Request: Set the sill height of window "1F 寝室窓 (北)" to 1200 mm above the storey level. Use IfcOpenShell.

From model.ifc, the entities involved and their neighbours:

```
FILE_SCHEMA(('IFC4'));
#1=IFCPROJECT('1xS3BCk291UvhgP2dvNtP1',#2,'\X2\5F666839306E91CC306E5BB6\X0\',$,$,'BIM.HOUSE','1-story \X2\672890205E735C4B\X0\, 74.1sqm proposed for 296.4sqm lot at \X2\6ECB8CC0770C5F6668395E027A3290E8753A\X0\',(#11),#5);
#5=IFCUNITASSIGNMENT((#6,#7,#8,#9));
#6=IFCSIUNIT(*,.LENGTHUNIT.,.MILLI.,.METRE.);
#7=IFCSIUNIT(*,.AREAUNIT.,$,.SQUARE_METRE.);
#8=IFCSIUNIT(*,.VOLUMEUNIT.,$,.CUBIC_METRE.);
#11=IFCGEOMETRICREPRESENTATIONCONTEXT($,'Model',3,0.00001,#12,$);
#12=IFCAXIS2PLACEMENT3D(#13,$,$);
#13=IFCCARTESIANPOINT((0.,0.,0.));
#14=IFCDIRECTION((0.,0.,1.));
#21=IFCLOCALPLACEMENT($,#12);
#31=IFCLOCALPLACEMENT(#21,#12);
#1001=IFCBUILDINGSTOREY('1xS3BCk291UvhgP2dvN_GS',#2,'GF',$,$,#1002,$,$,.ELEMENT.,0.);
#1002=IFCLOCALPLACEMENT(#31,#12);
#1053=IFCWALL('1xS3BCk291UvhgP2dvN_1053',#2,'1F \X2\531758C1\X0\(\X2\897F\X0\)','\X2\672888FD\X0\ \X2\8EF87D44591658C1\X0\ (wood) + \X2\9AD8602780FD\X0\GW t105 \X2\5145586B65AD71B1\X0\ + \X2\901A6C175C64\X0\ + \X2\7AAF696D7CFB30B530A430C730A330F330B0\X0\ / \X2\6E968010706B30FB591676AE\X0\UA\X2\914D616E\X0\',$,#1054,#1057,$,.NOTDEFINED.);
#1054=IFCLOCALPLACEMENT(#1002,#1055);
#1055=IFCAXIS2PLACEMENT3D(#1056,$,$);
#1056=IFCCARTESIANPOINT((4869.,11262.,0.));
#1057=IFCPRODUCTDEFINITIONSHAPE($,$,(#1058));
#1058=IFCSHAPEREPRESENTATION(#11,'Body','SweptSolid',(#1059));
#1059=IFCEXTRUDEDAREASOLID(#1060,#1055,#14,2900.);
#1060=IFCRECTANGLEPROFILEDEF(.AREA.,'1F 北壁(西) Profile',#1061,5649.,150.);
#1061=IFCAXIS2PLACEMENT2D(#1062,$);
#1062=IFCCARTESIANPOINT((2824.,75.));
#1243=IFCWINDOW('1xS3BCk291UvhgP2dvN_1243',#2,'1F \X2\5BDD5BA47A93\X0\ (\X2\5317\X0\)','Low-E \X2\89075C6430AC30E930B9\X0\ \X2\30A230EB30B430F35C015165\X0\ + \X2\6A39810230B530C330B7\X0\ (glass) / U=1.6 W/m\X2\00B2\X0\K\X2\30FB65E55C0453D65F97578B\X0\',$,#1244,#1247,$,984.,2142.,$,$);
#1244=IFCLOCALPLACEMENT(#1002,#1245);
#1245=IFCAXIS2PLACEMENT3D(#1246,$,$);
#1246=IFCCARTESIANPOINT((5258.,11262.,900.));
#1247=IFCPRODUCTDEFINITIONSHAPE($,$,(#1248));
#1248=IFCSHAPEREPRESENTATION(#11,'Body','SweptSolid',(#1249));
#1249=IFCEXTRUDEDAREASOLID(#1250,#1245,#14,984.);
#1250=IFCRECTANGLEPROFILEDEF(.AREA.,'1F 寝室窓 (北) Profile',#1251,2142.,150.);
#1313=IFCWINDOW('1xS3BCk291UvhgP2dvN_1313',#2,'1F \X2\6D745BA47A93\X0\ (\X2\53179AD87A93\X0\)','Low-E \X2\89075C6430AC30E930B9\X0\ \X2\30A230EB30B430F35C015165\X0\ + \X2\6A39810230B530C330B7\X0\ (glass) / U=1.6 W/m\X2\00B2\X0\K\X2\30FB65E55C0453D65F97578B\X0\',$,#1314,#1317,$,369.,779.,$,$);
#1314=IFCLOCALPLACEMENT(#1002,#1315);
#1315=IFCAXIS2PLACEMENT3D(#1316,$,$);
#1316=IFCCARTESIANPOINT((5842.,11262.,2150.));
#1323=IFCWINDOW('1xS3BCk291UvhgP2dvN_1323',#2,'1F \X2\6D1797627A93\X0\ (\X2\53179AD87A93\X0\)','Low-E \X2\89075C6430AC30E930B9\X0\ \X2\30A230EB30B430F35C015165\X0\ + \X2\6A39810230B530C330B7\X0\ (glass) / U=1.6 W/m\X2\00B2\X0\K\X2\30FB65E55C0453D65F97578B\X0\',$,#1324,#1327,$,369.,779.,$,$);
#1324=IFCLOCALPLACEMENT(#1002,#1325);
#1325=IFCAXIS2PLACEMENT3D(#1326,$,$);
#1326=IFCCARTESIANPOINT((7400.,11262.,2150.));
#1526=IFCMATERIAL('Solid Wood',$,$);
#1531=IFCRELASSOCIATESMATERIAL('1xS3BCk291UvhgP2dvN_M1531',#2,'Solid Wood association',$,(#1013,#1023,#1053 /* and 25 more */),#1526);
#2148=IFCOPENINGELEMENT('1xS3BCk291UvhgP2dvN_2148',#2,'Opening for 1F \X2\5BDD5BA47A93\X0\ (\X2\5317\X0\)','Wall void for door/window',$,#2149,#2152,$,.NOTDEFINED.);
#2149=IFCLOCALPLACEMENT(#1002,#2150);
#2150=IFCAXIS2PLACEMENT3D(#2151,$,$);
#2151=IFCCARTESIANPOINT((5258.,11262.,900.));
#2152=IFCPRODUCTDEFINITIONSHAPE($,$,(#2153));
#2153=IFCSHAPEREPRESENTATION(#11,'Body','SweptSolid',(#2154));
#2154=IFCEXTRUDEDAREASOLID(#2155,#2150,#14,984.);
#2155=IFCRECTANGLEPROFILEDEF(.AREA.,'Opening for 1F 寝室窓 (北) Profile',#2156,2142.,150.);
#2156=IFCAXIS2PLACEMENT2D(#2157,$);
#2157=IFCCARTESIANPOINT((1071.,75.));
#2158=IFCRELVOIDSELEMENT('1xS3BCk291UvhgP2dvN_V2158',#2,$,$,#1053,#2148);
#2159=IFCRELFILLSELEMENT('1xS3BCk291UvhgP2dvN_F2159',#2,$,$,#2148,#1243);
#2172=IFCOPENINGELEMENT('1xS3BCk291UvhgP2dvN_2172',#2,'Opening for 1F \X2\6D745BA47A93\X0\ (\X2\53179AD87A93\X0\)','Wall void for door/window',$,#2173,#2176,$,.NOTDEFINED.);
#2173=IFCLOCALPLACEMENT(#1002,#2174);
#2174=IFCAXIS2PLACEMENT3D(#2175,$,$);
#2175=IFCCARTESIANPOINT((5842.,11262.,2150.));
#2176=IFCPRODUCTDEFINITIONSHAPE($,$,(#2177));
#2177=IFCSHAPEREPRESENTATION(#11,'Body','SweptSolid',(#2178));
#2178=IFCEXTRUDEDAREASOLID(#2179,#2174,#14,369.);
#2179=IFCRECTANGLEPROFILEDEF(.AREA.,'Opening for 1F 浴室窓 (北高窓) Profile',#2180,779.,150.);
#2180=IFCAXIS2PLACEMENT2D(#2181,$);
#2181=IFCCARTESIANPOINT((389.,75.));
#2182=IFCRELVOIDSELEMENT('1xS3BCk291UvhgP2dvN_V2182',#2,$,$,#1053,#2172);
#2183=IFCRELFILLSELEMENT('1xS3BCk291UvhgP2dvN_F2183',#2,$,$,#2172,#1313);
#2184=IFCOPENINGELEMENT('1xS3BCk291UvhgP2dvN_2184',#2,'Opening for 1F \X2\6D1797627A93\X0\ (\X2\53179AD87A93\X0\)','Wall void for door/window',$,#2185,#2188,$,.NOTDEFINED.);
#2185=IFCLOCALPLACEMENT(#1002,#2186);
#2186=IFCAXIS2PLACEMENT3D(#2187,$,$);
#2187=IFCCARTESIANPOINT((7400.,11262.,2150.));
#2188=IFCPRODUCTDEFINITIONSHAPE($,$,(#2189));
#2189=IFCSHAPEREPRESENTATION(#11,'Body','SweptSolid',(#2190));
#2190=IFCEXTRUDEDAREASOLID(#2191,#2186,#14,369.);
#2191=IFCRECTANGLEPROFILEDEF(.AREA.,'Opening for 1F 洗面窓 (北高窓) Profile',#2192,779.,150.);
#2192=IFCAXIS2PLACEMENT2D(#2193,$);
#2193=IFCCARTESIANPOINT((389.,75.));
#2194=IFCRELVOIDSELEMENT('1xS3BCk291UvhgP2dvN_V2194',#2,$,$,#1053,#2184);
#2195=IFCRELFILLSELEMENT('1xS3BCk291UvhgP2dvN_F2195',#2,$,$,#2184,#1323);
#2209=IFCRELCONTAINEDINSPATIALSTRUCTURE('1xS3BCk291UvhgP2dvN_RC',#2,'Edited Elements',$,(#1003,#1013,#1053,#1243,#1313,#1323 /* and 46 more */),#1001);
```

```python
import numpy as np
import ifcopenshell
import ifcopenshell.api.geometry
import ifcopenshell.geom
import ifcopenshell.util.element
import ifcopenshell.util.placement
import ifcopenshell.util.shape
import ifcopenshell.util.unit

model = ifcopenshell.open("model.ifc")
unit_scale = ifcopenshell.util.unit.calculate_unit_scale(model)

window = model.by_id(1243)
opening = window.FillsVoids[0].RelatingOpeningElement
storey = ifcopenshell.util.element.get_container(window, ifc_class="IfcBuildingStorey")
level = ifcopenshell.util.placement.get_local_placement(storey.ObjectPlacement)[2, 3]

# The opening's origin need not be at the sill, so measure its lowest point.
shape = ifcopenshell.geom.create_shape(ifcopenshell.geom.settings(), opening)
bottom = ifcopenshell.util.shape.get_shape_bottom_elevation(shape, shape.geometry) / unit_scale
dz = level + 1.2 / unit_scale - bottom

shift = np.array([0.0, 0.0, dz])
# The window is not placed relative to its opening, so move both.
for product in (opening, window):
    matrix = ifcopenshell.util.placement.get_local_placement(product.ObjectPlacement)
    matrix[:3, 3] += shift
    ifcopenshell.api.geometry.edit_object_placement(model, product=product, matrix=matrix, is_si=False)

print(f"moved by {dz * unit_scale:+.3f} m")

model.write("model_updated.ifc")
```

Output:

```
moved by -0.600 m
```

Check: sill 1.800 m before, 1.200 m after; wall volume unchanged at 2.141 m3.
